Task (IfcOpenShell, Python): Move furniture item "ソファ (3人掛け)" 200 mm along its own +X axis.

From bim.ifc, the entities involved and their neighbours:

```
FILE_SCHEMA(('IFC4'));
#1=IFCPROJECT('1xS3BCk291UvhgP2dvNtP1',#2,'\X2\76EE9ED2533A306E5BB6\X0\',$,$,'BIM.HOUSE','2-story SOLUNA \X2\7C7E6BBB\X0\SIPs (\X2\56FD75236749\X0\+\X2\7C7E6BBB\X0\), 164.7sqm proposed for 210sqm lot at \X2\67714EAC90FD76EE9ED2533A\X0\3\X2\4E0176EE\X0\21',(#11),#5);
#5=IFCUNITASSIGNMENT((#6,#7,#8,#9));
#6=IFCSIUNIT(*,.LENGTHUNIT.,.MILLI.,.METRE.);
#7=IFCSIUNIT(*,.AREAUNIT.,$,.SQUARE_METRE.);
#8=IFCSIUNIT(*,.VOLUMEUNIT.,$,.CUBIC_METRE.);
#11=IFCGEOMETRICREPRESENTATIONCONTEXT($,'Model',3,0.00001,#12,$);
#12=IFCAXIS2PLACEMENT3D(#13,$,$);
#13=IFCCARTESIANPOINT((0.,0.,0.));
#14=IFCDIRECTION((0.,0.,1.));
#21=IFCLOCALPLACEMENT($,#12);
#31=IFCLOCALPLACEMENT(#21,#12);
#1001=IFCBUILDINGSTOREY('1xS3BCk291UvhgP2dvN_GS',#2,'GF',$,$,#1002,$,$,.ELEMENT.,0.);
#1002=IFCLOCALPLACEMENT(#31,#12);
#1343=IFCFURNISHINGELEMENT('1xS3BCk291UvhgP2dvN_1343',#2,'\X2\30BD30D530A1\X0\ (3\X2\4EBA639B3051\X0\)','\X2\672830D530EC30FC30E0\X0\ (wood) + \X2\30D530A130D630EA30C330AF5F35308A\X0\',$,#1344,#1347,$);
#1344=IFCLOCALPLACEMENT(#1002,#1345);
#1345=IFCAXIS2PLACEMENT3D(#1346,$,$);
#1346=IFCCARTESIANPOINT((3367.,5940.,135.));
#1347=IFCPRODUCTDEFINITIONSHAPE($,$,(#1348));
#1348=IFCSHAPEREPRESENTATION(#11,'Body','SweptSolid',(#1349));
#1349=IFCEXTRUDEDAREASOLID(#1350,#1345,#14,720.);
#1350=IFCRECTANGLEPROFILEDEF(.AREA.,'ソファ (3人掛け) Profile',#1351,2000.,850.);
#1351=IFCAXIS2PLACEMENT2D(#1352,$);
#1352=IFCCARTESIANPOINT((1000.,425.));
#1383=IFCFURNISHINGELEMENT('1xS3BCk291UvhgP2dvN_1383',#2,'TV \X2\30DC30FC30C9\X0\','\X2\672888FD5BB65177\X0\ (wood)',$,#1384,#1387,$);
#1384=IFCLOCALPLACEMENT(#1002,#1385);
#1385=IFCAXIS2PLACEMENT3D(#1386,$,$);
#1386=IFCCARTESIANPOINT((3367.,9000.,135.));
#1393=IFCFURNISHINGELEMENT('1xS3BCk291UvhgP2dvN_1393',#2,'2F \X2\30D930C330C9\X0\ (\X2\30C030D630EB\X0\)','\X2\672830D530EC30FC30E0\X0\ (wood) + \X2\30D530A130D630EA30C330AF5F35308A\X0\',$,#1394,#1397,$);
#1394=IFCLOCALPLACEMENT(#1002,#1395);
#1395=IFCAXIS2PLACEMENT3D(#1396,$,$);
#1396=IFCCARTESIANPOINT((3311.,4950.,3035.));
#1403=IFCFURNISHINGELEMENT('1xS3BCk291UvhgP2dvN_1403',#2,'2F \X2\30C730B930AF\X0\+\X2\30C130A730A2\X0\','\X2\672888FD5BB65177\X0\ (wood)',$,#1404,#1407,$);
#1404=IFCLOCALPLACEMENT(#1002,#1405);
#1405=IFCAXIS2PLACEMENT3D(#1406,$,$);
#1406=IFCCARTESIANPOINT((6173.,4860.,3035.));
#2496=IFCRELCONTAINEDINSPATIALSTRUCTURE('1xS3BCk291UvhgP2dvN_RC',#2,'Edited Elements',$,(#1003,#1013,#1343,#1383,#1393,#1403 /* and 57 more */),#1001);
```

```python
import ifcopenshell
import ifcopenshell.api.geometry
import ifcopenshell.util.placement
import ifcopenshell.util.unit

model = ifcopenshell.open("bim.ifc")
unit_scale = ifcopenshell.util.unit.calculate_unit_scale(model)

item = model.by_guid("1xS3BCk291UvhgP2dvN_1343")
matrix = ifcopenshell.util.placement.get_local_placement(item.ObjectPlacement)
matrix[:3, 3] += matrix[:3, 0] * 0.2 / unit_scale
ifcopenshell.api.geometry.edit_object_placement(model, product=item, matrix=matrix, is_si=False)

print(ifcopenshell.util.placement.get_local_placement(item.ObjectPlacement).round(3) + 0.0)

model.write("bim-out.ifc")
```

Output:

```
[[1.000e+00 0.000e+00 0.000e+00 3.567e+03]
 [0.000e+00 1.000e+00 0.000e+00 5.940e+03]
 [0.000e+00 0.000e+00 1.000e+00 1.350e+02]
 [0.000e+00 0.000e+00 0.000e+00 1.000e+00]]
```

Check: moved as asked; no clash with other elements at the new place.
